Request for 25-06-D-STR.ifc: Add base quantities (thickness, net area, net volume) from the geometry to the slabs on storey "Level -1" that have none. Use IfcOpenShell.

First a look at what the model holds.

```python
import ifcopenshell
import ifcopenshell.util.element
import ifcopenshell.util.unit

model = ifcopenshell.open("25-06-D-STR.ifc")
print(model.schema)
for unit_type in ("LENGTHUNIT", "AREAUNIT", "VOLUMEUNIT"):
    print(unit_type, ifcopenshell.util.unit.calculate_unit_scale(model, unit_type))
storey = next(s for s in model.by_type("IfcBuildingStorey") if s.Name == "Level -1")
slabs = [e for e in ifcopenshell.util.element.get_decomposition(storey) if e.is_a("IfcSlab")]
for e in sorted(slabs, key=lambda e: e.id()):
    print(e.id(), e.is_a(), e.Name, list(ifcopenshell.util.element.get_psets(e, qtos_only=True)), sep=" | ")
```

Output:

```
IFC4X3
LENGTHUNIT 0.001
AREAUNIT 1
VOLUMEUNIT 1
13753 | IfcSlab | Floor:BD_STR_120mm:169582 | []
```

```python
import ifcopenshell
import ifcopenshell.api.pset
import ifcopenshell.geom
import ifcopenshell.util.element
import ifcopenshell.util.shape
import ifcopenshell.util.unit

model = ifcopenshell.open("25-06-D-STR.ifc")
unit_scale = ifcopenshell.util.unit.calculate_unit_scale(model)
area_scale = ifcopenshell.util.unit.calculate_unit_scale(model, "AREAUNIT")
volume_scale = ifcopenshell.util.unit.calculate_unit_scale(model, "VOLUMEUNIT")
settings = ifcopenshell.geom.settings()

storey = next(s for s in model.by_type("IfcBuildingStorey") if s.Name == "Level -1")
slabs = [e for e in ifcopenshell.util.element.get_decomposition(storey) if e.is_a("IfcSlab")]

for e in sorted(slabs, key=lambda e: e.id()):
    if ifcopenshell.util.element.get_psets(e, qtos_only=True, should_inherit=False):
        continue
    # Geometry comes back in metres, in the element's own axes.
    shape = ifcopenshell.geom.create_shape(settings, e)
    values = {
        "Width": ifcopenshell.util.shape.get_z(shape.geometry) / unit_scale,
        "NetArea": ifcopenshell.util.shape.get_footprint_area(shape.geometry) / area_scale,
        "NetVolume": ifcopenshell.util.shape.get_volume(shape.geometry) / volume_scale,
    }
    qto = ifcopenshell.api.pset.add_qto(model, product=e, name="Qto_SlabBaseQuantities")
    ifcopenshell.api.pset.edit_qto(model, qto=qto, properties=values)
    print(e.id(), {k: round(v, 3) for k, v in values.items()})

model.write("25-06-D-STR_edited.ifc")
```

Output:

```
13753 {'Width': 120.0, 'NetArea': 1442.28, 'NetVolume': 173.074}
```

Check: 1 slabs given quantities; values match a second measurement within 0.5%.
